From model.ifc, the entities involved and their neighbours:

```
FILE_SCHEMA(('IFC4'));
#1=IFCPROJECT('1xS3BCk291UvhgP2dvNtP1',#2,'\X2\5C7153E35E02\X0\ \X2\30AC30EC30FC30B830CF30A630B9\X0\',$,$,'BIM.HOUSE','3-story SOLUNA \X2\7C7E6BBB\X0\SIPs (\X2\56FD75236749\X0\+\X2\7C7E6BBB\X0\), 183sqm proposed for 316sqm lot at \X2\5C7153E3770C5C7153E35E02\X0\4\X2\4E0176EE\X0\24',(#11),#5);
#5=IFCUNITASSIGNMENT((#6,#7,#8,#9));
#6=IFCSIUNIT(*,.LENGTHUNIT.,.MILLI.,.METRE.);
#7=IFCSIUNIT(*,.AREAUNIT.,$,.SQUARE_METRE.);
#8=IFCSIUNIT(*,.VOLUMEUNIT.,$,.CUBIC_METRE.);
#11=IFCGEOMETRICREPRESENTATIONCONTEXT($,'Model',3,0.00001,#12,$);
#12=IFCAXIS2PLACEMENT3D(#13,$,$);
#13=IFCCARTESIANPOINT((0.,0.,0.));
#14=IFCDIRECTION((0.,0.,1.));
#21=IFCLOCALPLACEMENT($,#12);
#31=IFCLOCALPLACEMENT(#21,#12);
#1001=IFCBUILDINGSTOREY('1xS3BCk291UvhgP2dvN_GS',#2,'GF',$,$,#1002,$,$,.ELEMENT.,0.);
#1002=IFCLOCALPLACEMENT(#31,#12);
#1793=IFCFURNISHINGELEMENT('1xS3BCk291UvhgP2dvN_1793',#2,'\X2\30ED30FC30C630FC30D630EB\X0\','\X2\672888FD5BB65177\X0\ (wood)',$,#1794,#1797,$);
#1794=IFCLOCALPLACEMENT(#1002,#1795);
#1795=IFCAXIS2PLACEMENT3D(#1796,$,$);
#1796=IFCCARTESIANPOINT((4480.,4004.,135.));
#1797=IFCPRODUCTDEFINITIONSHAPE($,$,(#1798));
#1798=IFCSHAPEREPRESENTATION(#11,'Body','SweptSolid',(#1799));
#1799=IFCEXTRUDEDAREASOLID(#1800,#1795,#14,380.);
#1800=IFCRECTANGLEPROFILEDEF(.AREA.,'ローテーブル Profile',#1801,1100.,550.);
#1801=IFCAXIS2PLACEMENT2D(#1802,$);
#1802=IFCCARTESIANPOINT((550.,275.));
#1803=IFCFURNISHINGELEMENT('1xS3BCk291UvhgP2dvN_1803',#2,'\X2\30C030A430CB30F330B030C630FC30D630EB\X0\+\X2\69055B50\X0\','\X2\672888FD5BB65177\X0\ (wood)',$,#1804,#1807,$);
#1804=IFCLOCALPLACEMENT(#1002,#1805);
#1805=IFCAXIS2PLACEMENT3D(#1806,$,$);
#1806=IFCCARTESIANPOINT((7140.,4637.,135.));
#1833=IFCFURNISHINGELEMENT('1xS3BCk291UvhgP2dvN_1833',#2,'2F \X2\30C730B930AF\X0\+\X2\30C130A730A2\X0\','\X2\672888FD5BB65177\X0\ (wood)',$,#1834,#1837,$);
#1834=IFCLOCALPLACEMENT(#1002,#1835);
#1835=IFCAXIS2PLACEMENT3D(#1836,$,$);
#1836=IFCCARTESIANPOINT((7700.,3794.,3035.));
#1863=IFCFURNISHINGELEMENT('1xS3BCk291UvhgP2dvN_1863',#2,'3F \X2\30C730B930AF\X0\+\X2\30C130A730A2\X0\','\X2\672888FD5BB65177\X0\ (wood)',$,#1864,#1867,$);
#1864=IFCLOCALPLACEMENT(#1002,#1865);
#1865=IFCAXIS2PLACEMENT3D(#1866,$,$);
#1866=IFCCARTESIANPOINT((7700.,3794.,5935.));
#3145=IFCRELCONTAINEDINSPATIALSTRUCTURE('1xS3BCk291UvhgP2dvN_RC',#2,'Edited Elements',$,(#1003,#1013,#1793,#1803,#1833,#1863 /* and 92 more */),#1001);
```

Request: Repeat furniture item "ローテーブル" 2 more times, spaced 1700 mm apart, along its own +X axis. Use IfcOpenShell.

```python
import ifcopenshell
import ifcopenshell.api.geometry
import ifcopenshell.api.root
import ifcopenshell.util.element
import ifcopenshell.util.placement
import ifcopenshell.util.unit

model = ifcopenshell.open("model.ifc")
unit_scale = ifcopenshell.util.unit.calculate_unit_scale(model)


def reuse_history(source, copy):
    """copy_class also copies each property set's owner history, people and application; keep the originals."""
    for rel in copy.IsDefinedBy:
        if rel.is_a("IfcRelDefinesByProperties") and (history := rel.RelatingPropertyDefinition.OwnerHistory):
            rel.RelatingPropertyDefinition.OwnerHistory = source.OwnerHistory
            ifcopenshell.util.element.remove_deep2(model, history)


source = model.by_id(1793)
base = ifcopenshell.util.placement.get_local_placement(source.ObjectPlacement)
step = base[:3, 0] * 1.7 / unit_scale

for i in range(1, 3):
    copy = ifcopenshell.api.root.copy_class(model, product=source)
    copy.Representation = ifcopenshell.util.element.copy_deep(
        model, source.Representation, exclude=["IfcGeometricRepresentationContext", "IfcRepresentationMap"]
    )
    reuse_history(source, copy)
    matrix = base.copy()
    matrix[:3, 3] += i * step
    print("added at", matrix[:3, 3].round(3) + 0.0)
    ifcopenshell.api.geometry.edit_object_placement(model, product=copy, matrix=matrix, is_si=False)

model.write("model_updated.ifc")
```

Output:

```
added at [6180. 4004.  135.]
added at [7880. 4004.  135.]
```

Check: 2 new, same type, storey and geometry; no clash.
